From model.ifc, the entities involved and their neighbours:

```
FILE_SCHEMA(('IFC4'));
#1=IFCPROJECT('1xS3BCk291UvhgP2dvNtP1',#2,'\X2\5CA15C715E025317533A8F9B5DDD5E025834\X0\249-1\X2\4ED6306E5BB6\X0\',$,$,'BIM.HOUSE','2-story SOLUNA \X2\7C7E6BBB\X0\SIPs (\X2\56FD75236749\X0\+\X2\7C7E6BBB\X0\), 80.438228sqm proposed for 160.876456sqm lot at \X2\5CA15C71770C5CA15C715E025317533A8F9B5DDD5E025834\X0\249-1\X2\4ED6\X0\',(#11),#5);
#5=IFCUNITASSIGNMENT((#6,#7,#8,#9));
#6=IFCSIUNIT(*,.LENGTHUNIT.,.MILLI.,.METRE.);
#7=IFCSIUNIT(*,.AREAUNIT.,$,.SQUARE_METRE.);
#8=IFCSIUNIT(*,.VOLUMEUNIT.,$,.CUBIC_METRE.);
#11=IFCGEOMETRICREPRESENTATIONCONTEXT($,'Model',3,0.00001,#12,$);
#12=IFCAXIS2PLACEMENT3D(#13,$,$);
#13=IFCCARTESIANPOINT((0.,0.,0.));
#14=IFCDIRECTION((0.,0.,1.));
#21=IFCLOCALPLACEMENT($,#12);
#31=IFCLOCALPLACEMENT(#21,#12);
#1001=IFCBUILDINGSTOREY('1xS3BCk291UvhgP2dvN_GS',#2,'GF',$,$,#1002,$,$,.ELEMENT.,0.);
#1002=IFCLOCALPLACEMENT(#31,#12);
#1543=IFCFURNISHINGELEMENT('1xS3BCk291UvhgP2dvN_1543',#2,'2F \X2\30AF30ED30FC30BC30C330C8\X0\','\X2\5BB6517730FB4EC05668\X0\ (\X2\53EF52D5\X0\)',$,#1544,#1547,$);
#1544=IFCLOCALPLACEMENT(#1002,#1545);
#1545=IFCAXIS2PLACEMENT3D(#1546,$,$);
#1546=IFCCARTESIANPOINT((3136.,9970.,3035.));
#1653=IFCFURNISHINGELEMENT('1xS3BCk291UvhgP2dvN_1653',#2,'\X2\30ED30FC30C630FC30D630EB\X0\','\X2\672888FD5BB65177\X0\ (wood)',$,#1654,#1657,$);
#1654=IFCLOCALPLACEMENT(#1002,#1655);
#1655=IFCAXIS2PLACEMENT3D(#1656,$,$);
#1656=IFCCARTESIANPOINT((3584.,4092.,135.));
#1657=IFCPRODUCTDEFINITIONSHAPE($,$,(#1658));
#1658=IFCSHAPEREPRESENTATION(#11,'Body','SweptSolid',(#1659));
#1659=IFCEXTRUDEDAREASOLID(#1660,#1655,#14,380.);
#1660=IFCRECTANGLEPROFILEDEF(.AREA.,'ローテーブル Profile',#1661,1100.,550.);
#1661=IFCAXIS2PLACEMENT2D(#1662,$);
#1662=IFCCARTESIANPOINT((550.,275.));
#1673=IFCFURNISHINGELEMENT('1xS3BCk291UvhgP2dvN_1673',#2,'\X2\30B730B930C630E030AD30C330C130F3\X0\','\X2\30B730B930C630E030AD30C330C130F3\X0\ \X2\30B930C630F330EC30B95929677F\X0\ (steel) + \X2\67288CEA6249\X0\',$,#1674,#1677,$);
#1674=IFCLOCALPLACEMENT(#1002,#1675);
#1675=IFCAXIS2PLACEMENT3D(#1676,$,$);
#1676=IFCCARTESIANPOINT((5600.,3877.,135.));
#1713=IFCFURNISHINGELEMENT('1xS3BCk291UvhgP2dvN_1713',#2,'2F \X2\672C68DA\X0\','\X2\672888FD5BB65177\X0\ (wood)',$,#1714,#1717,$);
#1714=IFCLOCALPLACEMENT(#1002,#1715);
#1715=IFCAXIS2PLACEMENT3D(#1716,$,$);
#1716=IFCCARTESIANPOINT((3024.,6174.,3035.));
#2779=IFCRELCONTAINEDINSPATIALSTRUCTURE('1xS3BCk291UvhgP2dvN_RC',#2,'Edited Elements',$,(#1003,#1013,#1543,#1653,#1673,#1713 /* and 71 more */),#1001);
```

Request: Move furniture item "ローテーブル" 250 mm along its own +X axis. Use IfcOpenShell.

```python
import ifcopenshell
import ifcopenshell.api.geometry
import ifcopenshell.util.placement

model = ifcopenshell.open("model.ifc")

item = model.by_id(1653)
matrix = ifcopenshell.util.placement.get_local_placement(item.ObjectPlacement)
matrix[:3, 3] += matrix[:3, 0] * 250.0
ifcopenshell.api.geometry.edit_object_placement(model, product=item, matrix=matrix, is_si=False)

print(ifcopenshell.util.placement.get_local_placement(item.ObjectPlacement).round(3) + 0.0)

model.write("model_rev.ifc")
```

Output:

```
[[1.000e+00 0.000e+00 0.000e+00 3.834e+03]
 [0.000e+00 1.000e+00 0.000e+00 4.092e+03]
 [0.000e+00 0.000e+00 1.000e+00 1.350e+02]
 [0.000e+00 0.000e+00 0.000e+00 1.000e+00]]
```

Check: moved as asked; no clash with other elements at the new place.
